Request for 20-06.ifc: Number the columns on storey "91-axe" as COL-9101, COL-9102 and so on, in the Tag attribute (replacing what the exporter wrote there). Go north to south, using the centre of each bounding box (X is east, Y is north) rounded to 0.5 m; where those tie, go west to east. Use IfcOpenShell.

First a look at what the model holds.

```python
import ifcopenshell
import ifcopenshell.util.element
import ifcopenshell.util.placement

model = ifcopenshell.open("20-06.ifc")
print(model.schema)
storey = next(s for s in model.by_type("IfcBuildingStorey") if s.Name == "91-axe")
columns = [e for e in ifcopenshell.util.element.get_decomposition(storey) if e.is_a("IfcColumn")]
for e in sorted(columns, key=lambda e: e.id()):
    origin = ifcopenshell.util.placement.get_local_placement(e.ObjectPlacement)[:3, 3]
    print(e.id(), e.Tag, e.Name, origin.round(2) + 0.0, sep=" | ")
```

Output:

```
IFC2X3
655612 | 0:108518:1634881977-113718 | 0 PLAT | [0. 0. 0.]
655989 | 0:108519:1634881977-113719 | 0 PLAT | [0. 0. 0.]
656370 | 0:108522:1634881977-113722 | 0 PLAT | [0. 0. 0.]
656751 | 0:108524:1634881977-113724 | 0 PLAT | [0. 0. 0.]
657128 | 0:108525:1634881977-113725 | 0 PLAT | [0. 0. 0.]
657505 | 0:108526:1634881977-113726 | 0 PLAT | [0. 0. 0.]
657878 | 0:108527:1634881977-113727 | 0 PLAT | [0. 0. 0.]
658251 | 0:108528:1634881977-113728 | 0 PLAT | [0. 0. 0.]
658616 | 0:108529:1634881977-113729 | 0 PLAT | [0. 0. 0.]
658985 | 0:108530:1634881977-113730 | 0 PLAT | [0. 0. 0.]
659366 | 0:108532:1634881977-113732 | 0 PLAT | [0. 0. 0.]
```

```python
import ifcopenshell
import ifcopenshell.geom
import ifcopenshell.util.element
import ifcopenshell.util.shape

model = ifcopenshell.open("20-06.ifc")
settings = ifcopenshell.geom.settings()
settings.set("use-world-coords", True)


def centre(element):
    shape = ifcopenshell.geom.create_shape(settings, element)
    return ifcopenshell.util.shape.get_bbox_centroid(shape.geometry)


storey = next(s for s in model.by_type("IfcBuildingStorey") if s.Name == "91-axe")
columns = [e for e in ifcopenshell.util.element.get_decomposition(storey) if e.is_a("IfcColumn")]

# Insertion points can sit at a corner or the storey origin, so sort by the geometry (in metres).
centres = {e: centre(e) for e in columns}
columns.sort(key=lambda e: (-round(centres[e][1] / 0.5), centres[e][0]))

for i, e in enumerate(columns, start=1):
    number = f"COL-91{i:02d}"
    e.Tag = number
    print(e.id(), number)

model.write("20-06-out.ifc")
```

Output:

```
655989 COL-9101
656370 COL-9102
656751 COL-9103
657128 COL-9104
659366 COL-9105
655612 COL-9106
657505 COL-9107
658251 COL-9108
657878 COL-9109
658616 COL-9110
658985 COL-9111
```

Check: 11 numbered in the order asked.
